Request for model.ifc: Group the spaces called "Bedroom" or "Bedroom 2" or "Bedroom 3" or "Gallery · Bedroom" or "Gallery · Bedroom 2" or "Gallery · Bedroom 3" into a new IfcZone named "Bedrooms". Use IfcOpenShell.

First a look at what the model holds.

```python
import ifcopenshell

model = ifcopenshell.open("model.ifc")
print(model.schema)
seen = {}
for space in model.by_type("IfcSpace"):
    seen[space.Name] = seen.get(space.Name, 0) + 1
for name, count in sorted(seen.items(), key=str):
    print(count, "x", name)
print("zones:", [z.Name for z in model.by_type("IfcZone")][:20])
```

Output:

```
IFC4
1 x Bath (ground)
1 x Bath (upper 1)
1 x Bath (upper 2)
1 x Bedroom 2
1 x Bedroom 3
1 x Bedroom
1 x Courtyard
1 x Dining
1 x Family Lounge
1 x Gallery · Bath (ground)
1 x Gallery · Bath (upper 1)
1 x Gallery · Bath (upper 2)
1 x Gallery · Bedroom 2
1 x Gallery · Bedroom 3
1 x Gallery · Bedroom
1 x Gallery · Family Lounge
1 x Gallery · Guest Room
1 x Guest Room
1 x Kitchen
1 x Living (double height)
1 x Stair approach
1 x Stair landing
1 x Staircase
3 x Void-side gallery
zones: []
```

```python
import ifcopenshell
import ifcopenshell.api.group
import ifcopenshell.api.root

model = ifcopenshell.open("model.ifc")

names = {"Bedroom", "Bedroom 2", "Bedroom 3", "Gallery · Bedroom", "Gallery · Bedroom 2", "Gallery · Bedroom 3"}
spaces = [s for s in model.by_type("IfcSpace") if s.Name in names]

zone = ifcopenshell.api.root.create_entity(model, ifc_class="IfcZone", name="Bedrooms")
ifcopenshell.api.group.assign_group(model, products=spaces, group=zone)
print(len(spaces), "spaces in", zone.Name)

model.write("model_updated.ifc")
```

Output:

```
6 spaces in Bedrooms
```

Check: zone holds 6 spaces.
